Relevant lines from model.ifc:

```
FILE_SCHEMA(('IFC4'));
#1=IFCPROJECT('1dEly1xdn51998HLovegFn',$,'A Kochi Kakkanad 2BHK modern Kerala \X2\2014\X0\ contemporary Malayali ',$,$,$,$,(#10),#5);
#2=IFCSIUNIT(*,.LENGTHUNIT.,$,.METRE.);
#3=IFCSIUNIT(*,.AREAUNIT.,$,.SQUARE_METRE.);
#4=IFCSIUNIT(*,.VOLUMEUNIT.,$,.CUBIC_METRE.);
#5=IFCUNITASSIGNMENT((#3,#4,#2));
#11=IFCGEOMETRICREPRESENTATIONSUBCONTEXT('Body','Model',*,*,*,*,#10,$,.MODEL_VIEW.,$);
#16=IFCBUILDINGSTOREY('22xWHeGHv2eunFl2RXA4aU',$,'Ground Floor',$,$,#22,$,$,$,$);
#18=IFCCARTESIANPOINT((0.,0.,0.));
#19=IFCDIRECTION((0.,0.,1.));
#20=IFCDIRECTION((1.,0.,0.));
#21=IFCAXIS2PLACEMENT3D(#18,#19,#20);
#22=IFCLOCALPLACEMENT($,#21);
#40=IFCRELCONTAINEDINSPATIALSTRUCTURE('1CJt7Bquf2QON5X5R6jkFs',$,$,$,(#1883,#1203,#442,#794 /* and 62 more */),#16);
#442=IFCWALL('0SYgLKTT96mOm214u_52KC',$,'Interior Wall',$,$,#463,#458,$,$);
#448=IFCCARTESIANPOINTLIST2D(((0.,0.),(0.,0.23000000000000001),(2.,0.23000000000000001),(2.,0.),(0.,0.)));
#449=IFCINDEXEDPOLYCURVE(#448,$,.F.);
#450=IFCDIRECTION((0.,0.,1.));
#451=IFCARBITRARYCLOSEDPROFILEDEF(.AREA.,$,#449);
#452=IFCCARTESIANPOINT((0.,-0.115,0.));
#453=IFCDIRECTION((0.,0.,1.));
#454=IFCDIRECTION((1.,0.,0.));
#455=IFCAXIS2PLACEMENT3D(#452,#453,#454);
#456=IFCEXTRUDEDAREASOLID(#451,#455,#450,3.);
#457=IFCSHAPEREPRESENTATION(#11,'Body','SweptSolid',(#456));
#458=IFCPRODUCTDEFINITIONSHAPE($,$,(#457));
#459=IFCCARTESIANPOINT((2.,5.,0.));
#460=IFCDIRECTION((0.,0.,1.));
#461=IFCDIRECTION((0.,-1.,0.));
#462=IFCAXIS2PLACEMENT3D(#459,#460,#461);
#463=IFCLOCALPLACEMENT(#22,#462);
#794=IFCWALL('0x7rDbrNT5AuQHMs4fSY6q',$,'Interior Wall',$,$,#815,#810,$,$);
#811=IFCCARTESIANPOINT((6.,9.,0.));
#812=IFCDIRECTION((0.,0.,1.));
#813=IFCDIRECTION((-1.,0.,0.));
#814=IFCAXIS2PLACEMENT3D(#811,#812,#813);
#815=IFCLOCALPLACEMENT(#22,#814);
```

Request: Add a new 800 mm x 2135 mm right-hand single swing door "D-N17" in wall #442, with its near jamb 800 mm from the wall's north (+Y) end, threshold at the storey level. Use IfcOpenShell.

```python
import numpy as np
import ifcopenshell
import ifcopenshell.api.feature
import ifcopenshell.api.geometry
import ifcopenshell.api.root
import ifcopenshell.api.spatial
import ifcopenshell.geom
import ifcopenshell.util.element
import ifcopenshell.util.placement
import ifcopenshell.util.representation
import ifcopenshell.util.shape
import ifcopenshell.util.unit

model = ifcopenshell.open("model.ifc")
unit_scale = ifcopenshell.util.unit.calculate_unit_scale(model)
settings = ifcopenshell.geom.settings()


def volume(element):
    """Net volume in cubic metres, openings subtracted."""
    shape = ifcopenshell.geom.create_shape(settings, element)
    return ifcopenshell.util.shape.get_volume(shape.geometry)


wall = model.by_guid("0SYgLKTT96mOm214u_52KC")
storey = ifcopenshell.util.element.get_container(wall, ifc_class="IfcBuildingStorey")
context = ifcopenshell.util.representation.get_context(model, "Model", "Body", "MODEL_VIEW")
before = volume(wall)

width, height, from_end, sill = 0.8, 2.135, 0.8, 0.0  # metres

# The wall runs along its own X axis, and the end named is its -X end.
wall_shape = ifcopenshell.geom.create_shape(settings, wall)
x, y, z = ifcopenshell.util.shape.get_vertices(wall_shape.geometry).T
start = x.min() + from_end
face, thickness = float(y.min()), float(y.max() - y.min())
wall_matrix = ifcopenshell.util.placement.get_local_placement(wall.ObjectPlacement)
level = ifcopenshell.util.placement.get_local_placement(storey.ObjectPlacement)[2, 3]


def in_wall(x, y):
    """Placement at x, y metres in the wall's axes, at sill height."""
    matrix = wall_matrix.copy()
    matrix[:, 3] = wall_matrix @ np.array([x / unit_scale, y / unit_scale, 0.0, 1.0])
    matrix[2, 3] = level + sill / unit_scale
    return matrix


# Opening: a box that overshoots both wall faces by 50 mm.
opening = ifcopenshell.api.root.create_entity(model, ifc_class="IfcOpeningElement", predefined_type="OPENING")
box = ifcopenshell.api.geometry.add_wall_representation(
    model, context=context, length=width, height=height, thickness=thickness + 0.1
)
ifcopenshell.api.geometry.assign_representation(model, product=opening, representation=box)
ifcopenshell.api.geometry.edit_object_placement(model, product=opening, matrix=in_wall(start, face - 0.05), is_si=False)
ifcopenshell.api.feature.add_feature(model, feature=opening, element=wall)

door = ifcopenshell.api.root.create_entity(model, ifc_class="IfcDoor", name="D-N17", predefined_type="DOOR")
door.OverallWidth, door.OverallHeight = width / unit_scale, height / unit_scale
door.OperationType = "SINGLE_SWING_RIGHT"
body = ifcopenshell.api.geometry.add_door_representation(
    model,
    context=context,
    overall_width=door.OverallWidth,
    overall_height=door.OverallHeight,
    operation_type="SINGLE_SWING_RIGHT",
    lining_properties={"LiningDepth": thickness / unit_scale, "ThresholdDepth": thickness / unit_scale},
)
ifcopenshell.api.geometry.assign_representation(model, product=door, representation=body)
ifcopenshell.api.spatial.assign_container(model, products=[door], relating_structure=storey)
ifcopenshell.api.feature.add_filling(model, opening=opening, element=door)

# The lining spans the wall, so the door starts at the wall face.
ifcopenshell.api.geometry.edit_object_placement(model, product=door, matrix=in_wall(start, face), is_si=False)

after = volume(wall)

print(f"wall volume {before:.3f} -> {after:.3f} m3")

model.write("model_rev.ifc")
```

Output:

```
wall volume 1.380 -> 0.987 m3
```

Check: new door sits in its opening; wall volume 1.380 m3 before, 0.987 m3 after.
